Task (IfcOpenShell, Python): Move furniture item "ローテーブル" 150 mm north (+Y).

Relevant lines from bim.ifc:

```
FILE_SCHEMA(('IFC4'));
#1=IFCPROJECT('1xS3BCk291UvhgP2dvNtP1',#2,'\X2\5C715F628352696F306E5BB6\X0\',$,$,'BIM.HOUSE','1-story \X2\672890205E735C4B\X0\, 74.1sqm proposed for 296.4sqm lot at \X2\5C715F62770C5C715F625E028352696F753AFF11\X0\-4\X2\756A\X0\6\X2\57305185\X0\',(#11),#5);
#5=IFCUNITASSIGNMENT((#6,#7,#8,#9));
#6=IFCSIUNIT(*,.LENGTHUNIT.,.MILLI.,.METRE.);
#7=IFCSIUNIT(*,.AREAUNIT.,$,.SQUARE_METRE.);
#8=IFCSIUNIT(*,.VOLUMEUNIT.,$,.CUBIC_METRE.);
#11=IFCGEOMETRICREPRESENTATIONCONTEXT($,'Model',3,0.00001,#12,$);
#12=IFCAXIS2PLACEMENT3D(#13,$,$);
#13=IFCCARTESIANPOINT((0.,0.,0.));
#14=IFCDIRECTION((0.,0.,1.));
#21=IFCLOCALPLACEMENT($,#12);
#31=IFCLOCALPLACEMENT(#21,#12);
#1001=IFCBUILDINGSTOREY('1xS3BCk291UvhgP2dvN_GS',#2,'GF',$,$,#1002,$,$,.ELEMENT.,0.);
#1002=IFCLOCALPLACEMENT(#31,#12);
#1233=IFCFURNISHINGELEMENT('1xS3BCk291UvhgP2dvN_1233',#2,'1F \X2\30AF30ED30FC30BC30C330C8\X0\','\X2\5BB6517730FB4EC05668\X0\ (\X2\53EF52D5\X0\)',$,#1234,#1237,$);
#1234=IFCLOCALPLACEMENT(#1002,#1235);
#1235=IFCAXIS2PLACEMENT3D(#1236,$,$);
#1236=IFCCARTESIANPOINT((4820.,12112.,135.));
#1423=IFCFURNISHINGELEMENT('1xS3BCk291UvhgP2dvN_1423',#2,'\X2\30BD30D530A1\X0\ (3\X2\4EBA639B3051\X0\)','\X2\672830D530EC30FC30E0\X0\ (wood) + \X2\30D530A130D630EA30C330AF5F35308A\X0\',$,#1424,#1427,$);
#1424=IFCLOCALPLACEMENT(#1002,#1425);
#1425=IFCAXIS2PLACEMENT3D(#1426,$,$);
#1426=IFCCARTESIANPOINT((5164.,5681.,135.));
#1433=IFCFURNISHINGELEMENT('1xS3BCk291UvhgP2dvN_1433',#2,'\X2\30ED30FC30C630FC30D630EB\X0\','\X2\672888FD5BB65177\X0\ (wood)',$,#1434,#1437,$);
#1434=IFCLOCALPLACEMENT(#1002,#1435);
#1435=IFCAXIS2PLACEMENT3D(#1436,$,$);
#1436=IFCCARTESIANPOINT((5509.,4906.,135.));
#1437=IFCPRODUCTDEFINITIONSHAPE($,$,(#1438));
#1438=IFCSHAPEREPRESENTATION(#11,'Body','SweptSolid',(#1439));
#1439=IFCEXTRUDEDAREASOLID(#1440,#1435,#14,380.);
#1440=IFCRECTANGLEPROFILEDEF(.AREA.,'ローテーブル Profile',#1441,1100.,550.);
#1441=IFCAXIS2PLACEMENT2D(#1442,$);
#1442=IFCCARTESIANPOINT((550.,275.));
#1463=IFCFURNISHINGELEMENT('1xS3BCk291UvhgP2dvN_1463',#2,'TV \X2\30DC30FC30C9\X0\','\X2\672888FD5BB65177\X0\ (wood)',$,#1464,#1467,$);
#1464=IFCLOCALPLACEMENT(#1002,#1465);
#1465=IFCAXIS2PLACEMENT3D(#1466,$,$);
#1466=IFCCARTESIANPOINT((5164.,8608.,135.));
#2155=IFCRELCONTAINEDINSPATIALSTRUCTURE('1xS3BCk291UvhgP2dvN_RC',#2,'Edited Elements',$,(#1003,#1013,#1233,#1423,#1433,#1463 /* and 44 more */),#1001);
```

```python
import ifcopenshell
import ifcopenshell.api.geometry
import ifcopenshell.util.placement
import ifcopenshell.util.unit

model = ifcopenshell.open("bim.ifc")
unit_scale = ifcopenshell.util.unit.calculate_unit_scale(model)

item = model.by_guid("1xS3BCk291UvhgP2dvN_1433")
matrix = ifcopenshell.util.placement.get_local_placement(item.ObjectPlacement)
matrix[1, 3] += 0.15 / unit_scale
ifcopenshell.api.geometry.edit_object_placement(model, product=item, matrix=matrix, is_si=False)

print(ifcopenshell.util.placement.get_local_placement(item.ObjectPlacement).round(3) + 0.0)

model.write("bim-out.ifc")
```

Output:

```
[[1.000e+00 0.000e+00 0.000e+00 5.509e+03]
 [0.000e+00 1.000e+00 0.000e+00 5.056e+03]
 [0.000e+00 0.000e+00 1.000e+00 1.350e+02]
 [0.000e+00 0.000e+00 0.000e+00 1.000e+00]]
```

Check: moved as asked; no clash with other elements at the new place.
